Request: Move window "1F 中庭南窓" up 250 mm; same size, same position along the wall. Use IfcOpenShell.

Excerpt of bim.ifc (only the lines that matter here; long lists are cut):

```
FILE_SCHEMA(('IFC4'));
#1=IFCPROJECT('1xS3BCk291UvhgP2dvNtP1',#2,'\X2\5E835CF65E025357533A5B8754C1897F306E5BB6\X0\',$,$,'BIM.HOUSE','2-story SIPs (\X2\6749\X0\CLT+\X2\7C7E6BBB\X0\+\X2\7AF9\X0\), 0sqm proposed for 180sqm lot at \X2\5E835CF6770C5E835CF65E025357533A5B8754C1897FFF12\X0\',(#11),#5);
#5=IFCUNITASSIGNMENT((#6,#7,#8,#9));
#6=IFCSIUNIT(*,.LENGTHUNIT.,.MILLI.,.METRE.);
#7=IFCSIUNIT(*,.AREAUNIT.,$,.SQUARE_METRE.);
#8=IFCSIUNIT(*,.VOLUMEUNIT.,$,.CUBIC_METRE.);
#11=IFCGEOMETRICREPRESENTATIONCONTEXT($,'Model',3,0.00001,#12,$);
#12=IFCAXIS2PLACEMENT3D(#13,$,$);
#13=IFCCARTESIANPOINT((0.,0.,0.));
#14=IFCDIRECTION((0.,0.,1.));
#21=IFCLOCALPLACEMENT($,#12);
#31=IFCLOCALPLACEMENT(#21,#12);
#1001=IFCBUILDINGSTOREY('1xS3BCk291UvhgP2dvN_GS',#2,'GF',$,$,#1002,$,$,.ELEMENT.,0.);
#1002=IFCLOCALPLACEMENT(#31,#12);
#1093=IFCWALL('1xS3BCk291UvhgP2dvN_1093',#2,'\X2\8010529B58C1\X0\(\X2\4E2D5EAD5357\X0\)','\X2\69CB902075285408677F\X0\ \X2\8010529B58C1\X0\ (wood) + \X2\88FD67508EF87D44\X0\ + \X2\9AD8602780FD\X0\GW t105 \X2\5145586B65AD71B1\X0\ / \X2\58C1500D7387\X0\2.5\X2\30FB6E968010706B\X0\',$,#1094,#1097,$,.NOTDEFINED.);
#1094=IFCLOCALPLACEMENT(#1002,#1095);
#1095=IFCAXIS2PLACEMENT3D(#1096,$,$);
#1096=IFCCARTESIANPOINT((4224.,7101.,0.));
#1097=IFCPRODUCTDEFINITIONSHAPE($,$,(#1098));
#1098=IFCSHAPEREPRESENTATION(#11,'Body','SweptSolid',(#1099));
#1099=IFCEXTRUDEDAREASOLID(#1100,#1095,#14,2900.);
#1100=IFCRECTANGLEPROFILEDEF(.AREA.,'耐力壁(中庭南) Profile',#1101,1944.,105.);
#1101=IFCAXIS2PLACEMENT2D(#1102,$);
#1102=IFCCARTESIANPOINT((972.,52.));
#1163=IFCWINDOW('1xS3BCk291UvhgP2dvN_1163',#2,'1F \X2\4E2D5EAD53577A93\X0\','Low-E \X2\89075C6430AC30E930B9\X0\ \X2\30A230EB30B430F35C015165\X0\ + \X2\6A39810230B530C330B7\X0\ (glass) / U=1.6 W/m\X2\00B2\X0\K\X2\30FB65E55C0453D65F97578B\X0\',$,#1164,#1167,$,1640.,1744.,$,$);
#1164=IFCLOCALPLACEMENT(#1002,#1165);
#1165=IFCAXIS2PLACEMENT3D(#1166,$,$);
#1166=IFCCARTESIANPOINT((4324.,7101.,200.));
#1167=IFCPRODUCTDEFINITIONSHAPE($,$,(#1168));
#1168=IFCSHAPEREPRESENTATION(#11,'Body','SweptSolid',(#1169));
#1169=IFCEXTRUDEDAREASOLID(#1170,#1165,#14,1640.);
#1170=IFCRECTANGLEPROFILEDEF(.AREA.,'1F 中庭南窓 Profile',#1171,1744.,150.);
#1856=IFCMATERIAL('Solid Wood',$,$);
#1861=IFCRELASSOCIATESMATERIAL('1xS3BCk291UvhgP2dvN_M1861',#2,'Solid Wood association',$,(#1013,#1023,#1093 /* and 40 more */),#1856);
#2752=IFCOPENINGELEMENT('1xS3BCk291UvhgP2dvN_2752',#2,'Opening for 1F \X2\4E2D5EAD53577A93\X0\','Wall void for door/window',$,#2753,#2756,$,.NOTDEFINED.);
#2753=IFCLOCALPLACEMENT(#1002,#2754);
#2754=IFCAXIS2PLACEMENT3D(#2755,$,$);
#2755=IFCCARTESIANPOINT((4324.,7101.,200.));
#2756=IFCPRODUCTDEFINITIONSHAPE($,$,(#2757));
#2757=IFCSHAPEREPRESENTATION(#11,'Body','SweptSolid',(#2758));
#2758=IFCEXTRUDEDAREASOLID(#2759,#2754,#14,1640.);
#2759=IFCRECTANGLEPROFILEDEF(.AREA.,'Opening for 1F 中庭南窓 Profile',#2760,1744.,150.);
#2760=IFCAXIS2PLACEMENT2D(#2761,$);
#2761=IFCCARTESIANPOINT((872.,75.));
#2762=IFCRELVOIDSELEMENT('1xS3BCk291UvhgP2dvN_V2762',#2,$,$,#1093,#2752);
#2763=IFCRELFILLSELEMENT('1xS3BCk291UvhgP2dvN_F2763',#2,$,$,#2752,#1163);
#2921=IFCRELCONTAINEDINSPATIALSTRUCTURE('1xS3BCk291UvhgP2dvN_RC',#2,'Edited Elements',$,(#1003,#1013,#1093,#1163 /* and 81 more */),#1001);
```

```python
import numpy as np
import ifcopenshell
import ifcopenshell.api.geometry
import ifcopenshell.util.placement
import ifcopenshell.util.unit

model = ifcopenshell.open("bim.ifc")
unit_scale = ifcopenshell.util.unit.calculate_unit_scale(model)

window = model.by_guid("1xS3BCk291UvhgP2dvN_1163")
opening = window.FillsVoids[0].RelatingOpeningElement
dz = 250.0

shift = np.array([0.0, 0.0, dz])
# The window is not placed relative to its opening, so move both.
for product in (opening, window):
    matrix = ifcopenshell.util.placement.get_local_placement(product.ObjectPlacement)
    matrix[:3, 3] += shift
    ifcopenshell.api.geometry.edit_object_placement(model, product=product, matrix=matrix, is_si=False)

print(f"moved by {dz * unit_scale:+.3f} m")

model.write("bim-out.ifc")
```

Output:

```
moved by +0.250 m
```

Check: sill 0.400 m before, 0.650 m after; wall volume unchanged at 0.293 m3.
